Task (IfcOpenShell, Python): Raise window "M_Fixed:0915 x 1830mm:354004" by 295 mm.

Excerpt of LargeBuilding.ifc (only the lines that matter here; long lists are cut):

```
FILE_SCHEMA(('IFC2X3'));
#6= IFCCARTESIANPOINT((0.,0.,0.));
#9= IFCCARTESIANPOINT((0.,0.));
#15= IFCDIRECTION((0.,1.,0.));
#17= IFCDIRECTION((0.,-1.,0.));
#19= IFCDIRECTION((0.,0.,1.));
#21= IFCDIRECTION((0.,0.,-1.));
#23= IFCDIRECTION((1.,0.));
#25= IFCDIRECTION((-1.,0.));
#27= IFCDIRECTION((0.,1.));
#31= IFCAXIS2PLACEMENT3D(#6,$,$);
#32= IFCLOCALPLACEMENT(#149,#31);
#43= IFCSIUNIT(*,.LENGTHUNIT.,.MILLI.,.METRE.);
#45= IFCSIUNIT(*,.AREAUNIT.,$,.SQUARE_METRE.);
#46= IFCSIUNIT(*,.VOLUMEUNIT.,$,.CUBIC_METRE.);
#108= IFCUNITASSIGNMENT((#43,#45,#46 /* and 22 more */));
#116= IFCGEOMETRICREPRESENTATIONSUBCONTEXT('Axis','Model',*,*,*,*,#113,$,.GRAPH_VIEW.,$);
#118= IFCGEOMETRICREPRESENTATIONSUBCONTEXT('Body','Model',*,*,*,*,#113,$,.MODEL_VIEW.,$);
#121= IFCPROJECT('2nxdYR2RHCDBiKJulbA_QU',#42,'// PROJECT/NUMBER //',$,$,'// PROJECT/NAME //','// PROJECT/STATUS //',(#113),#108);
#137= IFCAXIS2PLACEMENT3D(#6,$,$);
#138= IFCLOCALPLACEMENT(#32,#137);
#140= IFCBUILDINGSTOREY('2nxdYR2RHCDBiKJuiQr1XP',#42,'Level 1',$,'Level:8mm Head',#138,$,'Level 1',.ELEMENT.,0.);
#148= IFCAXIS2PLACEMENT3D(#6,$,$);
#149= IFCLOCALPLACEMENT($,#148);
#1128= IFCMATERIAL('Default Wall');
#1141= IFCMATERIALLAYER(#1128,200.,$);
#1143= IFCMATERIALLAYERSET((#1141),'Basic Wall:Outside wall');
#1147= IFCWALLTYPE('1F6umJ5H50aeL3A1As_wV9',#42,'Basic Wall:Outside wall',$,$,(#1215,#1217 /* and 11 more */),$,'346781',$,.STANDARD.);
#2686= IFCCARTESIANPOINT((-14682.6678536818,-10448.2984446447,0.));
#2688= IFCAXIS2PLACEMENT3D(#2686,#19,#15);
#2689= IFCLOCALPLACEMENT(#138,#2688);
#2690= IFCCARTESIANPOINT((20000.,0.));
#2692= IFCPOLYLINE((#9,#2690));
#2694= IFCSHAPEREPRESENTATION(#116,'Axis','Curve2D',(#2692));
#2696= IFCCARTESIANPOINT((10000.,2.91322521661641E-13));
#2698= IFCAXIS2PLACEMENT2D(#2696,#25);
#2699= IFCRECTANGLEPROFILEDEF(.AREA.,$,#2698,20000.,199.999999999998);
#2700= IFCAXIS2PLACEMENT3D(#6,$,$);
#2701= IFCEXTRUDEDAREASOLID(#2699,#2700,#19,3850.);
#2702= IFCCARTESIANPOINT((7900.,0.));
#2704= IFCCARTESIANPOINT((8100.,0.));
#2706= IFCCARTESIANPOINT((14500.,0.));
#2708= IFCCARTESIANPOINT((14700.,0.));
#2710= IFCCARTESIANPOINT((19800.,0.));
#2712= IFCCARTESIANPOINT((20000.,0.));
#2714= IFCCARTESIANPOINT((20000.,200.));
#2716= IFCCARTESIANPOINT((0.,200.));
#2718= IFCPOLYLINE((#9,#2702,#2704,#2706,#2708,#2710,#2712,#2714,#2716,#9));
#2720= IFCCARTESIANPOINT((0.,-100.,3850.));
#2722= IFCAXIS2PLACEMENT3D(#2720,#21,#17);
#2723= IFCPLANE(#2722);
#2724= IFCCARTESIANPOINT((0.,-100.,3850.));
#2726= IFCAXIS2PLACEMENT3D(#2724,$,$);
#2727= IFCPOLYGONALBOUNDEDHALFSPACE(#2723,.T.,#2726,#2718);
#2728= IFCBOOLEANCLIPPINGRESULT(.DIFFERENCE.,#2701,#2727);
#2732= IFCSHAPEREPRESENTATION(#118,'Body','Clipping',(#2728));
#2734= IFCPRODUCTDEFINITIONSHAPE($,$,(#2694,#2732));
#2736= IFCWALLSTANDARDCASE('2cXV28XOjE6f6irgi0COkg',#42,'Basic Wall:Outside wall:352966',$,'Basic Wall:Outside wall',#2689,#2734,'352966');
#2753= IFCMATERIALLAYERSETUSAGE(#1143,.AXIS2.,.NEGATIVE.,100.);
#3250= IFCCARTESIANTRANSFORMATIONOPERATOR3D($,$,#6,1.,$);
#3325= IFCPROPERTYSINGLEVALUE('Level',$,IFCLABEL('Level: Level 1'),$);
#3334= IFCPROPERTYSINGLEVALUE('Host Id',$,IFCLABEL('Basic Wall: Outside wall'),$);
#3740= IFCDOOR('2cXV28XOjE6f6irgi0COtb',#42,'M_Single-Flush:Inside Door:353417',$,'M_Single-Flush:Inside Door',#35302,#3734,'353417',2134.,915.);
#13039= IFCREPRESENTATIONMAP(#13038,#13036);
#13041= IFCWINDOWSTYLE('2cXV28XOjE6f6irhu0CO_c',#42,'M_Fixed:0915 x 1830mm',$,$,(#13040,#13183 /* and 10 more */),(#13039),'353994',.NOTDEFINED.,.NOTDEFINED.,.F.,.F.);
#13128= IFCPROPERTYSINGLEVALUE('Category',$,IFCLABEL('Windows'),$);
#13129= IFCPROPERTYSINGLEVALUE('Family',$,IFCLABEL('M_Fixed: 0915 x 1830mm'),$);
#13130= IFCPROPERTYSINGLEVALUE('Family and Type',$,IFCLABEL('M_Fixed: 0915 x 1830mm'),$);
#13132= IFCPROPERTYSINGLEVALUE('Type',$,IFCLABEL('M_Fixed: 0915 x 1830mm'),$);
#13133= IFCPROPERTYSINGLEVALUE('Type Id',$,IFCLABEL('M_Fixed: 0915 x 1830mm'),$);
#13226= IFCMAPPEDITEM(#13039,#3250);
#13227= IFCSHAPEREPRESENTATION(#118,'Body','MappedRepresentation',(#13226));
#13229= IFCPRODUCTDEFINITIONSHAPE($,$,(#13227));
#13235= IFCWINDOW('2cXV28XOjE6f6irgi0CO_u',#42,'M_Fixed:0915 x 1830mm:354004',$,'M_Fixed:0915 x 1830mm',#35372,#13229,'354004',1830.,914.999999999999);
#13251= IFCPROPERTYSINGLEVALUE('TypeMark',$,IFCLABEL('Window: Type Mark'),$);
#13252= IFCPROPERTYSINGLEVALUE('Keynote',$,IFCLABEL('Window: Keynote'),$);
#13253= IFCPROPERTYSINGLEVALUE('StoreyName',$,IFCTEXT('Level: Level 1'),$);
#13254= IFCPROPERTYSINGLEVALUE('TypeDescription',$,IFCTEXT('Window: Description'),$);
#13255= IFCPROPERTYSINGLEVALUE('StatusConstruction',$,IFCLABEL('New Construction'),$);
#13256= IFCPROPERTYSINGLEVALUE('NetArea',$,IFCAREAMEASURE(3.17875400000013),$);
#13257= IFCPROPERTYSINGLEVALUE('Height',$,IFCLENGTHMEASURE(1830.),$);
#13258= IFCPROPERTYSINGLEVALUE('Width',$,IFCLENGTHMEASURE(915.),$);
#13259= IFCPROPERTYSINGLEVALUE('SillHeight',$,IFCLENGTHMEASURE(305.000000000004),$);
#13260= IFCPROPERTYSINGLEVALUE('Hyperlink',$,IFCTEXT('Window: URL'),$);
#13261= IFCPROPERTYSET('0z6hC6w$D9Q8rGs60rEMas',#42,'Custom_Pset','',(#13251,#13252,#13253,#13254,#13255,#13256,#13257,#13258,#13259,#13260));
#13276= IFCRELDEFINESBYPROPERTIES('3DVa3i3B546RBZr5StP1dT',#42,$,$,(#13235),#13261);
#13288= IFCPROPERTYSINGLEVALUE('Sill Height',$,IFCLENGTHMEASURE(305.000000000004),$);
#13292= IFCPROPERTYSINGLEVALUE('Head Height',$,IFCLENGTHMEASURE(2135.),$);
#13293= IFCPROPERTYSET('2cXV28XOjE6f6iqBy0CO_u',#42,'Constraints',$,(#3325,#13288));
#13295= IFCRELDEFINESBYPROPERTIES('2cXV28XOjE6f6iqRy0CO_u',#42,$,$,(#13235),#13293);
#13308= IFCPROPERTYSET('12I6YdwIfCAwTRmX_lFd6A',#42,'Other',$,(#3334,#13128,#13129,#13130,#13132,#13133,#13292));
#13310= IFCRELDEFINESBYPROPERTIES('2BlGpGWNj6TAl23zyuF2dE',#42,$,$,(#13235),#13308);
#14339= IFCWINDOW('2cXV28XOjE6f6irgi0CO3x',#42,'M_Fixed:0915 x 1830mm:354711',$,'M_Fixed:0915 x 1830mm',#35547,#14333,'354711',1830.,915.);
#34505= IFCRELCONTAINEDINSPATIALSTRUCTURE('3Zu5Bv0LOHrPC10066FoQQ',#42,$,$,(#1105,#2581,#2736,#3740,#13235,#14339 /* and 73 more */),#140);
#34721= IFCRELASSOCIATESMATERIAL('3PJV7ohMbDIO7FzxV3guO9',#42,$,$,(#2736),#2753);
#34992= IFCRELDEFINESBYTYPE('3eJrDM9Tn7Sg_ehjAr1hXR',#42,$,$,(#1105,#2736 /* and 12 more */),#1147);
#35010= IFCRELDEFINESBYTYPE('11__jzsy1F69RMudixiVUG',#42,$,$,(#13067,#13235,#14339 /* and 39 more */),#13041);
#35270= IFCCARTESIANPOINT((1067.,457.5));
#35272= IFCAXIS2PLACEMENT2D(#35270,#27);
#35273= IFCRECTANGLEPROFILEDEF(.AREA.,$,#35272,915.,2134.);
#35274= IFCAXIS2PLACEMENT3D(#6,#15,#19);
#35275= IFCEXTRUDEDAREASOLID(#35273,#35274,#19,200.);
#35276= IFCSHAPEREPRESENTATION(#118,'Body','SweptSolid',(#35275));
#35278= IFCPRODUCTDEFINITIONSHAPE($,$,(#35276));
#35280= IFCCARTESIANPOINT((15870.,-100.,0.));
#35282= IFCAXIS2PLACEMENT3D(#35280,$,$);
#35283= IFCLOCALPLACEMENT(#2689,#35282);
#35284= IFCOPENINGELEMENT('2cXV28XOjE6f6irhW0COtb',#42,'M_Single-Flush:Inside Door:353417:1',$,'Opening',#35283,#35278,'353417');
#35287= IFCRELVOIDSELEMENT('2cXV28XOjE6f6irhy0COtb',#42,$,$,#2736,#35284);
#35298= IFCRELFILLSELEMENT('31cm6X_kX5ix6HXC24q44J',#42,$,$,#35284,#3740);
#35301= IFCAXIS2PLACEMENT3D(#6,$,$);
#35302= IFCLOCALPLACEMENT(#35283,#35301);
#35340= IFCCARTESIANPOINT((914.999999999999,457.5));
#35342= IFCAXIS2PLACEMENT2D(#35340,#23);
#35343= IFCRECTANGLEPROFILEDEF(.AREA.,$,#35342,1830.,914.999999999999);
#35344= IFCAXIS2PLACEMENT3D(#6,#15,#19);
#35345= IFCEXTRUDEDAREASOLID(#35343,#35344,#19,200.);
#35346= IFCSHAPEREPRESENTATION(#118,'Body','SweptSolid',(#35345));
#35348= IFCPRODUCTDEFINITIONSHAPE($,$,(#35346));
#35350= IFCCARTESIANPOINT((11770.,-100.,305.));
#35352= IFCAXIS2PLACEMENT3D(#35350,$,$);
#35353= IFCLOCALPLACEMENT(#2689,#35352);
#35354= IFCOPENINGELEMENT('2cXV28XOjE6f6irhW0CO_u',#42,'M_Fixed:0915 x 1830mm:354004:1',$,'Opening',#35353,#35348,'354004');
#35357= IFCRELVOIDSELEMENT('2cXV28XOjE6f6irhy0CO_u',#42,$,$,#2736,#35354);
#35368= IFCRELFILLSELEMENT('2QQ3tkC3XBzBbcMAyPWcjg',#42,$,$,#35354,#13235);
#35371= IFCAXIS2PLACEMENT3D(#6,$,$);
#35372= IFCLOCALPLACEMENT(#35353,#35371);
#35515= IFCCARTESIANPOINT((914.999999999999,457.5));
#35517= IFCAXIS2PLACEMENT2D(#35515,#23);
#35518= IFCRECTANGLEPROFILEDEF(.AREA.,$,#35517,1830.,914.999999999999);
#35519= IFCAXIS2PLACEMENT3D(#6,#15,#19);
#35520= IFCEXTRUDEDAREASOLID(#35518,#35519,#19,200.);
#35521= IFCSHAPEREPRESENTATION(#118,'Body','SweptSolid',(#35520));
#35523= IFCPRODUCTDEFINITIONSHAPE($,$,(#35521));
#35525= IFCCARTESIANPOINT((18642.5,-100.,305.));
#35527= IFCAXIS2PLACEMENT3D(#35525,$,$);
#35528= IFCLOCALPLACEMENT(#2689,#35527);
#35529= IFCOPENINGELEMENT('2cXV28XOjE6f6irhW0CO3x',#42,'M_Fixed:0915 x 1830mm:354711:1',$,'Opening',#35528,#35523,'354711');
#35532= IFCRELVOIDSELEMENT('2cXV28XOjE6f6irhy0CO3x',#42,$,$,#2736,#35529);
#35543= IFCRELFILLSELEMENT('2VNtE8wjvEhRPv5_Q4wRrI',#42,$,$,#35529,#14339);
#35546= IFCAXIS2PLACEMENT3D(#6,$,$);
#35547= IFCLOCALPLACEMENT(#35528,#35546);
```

```python
import numpy as np
import ifcopenshell
import ifcopenshell.api.geometry
import ifcopenshell.api.pset
import ifcopenshell.util.element
import ifcopenshell.util.placement
import ifcopenshell.util.unit

model = ifcopenshell.open("LargeBuilding.ifc")
unit_scale = ifcopenshell.util.unit.calculate_unit_scale(model)

window = model.by_guid("2cXV28XOjE6f6irgi0CO_u")
opening = window.FillsVoids[0].RelatingOpeningElement
dz = 0.295 / unit_scale

shift = np.array([0.0, 0.0, dz])
# The window is placed relative to its opening, so it follows when the opening moves.
matrix = ifcopenshell.util.placement.get_local_placement(opening.ObjectPlacement)
matrix[:3, 3] += shift
ifcopenshell.api.geometry.edit_object_placement(
    model, product=opening, matrix=matrix, is_si=False, should_transform_children=True
)

# Keep the stored heights in step.
pset = model.by_id(ifcopenshell.util.element.get_pset(window, "Custom_Pset", should_inherit=False)["id"])
ifcopenshell.api.pset.edit_pset(model, pset=pset, properties={
    "SillHeight": model.create_entity("IfcLengthMeasure", ifcopenshell.util.element.get_pset(window, "Constraints", "Sill Height") + dz),
})
pset = model.by_id(ifcopenshell.util.element.get_pset(window, "Constraints", should_inherit=False)["id"])
ifcopenshell.api.pset.edit_pset(model, pset=pset, properties={
    "Sill Height": model.create_entity("IfcLengthMeasure", ifcopenshell.util.element.get_pset(window, "Constraints", "Sill Height") + dz),
})
pset = model.by_id(ifcopenshell.util.element.get_pset(window, "Other", should_inherit=False)["id"])
ifcopenshell.api.pset.edit_pset(model, pset=pset, properties={
    "Head Height": model.create_entity("IfcLengthMeasure", ifcopenshell.util.element.get_pset(window, "Other", "Head Height") + dz),
})

print(f"moved by {dz * unit_scale:+.3f} m")

model.write("LargeBuilding_edited.ifc")
```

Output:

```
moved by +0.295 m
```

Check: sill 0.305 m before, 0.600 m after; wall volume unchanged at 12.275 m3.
